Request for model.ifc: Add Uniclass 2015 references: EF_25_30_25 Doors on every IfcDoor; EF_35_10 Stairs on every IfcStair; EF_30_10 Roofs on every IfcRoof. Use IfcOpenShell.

First a look at what the model holds.

```python
import ifcopenshell

model = ifcopenshell.open("model.ifc")
print(model.schema)
print("classifications:", [c.Name for c in model.by_type("IfcClassification")])
for ifc_class in ("IfcDoor", "IfcRoof", "IfcStair", "IfcWall", "IfcWindow"):
    print(ifc_class, len(model.by_type(ifc_class)))
```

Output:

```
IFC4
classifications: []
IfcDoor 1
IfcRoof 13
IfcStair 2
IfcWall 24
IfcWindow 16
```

```python
import ifcopenshell
import ifcopenshell.api.classification

model = ifcopenshell.open("model.ifc")

system = ifcopenshell.api.classification.add_classification(model, classification="Uniclass 2015")

codes = {
    "IfcDoor": ("EF_25_30_25", "Doors"),
    "IfcStair": ("EF_35_10", "Stairs"),
    "IfcRoof": ("EF_30_10", "Roofs"),
}
for ifc_class, (code, name) in codes.items():
    products = model.by_type(ifc_class)
    ifcopenshell.api.classification.add_reference(
        model, products=products, classification=system, identification=code, name=name
    )
    print(code, len(products))

model.write("model_v2.ifc")
```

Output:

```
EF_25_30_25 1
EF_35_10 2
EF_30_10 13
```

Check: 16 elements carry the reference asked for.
